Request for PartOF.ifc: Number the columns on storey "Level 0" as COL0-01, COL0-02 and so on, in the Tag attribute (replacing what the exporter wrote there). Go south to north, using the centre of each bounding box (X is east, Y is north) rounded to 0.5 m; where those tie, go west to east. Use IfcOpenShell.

First a look at what the model holds.

```python
import ifcopenshell
import ifcopenshell.util.element
import ifcopenshell.util.placement

model = ifcopenshell.open("PartOF.ifc")
print(model.schema)
storey = next(s for s in model.by_type("IfcBuildingStorey") if s.Name == "Level 0")
columns = [e for e in ifcopenshell.util.element.get_decomposition(storey) if e.is_a("IfcColumn")]
for e in sorted(columns, key=lambda e: e.id()):
    origin = ifcopenshell.util.placement.get_local_placement(e.ObjectPlacement)[:3, 3]
    print(e.id(), e.Tag, e.Name, origin.round(2) + 0.0, sep=" | ")
```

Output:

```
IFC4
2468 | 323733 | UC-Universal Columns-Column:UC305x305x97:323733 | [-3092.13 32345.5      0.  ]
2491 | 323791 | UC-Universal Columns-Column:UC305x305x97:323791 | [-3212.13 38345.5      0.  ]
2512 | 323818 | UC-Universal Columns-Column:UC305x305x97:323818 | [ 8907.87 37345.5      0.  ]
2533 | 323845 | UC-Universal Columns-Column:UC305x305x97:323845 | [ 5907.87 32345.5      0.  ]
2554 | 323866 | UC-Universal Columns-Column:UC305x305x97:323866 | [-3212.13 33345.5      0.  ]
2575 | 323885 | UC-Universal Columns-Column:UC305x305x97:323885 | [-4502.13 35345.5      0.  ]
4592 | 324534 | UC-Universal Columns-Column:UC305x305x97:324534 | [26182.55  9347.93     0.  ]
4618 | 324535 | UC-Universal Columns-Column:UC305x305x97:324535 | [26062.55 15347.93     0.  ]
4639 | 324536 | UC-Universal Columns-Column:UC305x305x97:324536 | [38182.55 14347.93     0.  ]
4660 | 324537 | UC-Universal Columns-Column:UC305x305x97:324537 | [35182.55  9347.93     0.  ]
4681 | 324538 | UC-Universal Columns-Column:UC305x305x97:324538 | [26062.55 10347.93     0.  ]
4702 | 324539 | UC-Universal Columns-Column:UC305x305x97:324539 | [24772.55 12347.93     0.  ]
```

```python
import ifcopenshell
import ifcopenshell.geom
import ifcopenshell.util.element
import ifcopenshell.util.shape

model = ifcopenshell.open("PartOF.ifc")
settings = ifcopenshell.geom.settings()
settings.set("use-world-coords", True)


def centre(element):
    shape = ifcopenshell.geom.create_shape(settings, element)
    return ifcopenshell.util.shape.get_bbox_centroid(shape.geometry)


storey = next(s for s in model.by_type("IfcBuildingStorey") if s.Name == "Level 0")
columns = [e for e in ifcopenshell.util.element.get_decomposition(storey) if e.is_a("IfcColumn")]

# Insertion points can sit at a corner or the storey origin, so sort by the geometry (in metres).
centres = {e: centre(e) for e in columns}
columns.sort(key=lambda e: (round(centres[e][1] / 0.5), centres[e][0]))

for i, e in enumerate(columns, start=1):
    number = f"COL0-{i:02d}"
    e.Tag = number
    print(e.id(), number)

model.write("PartOF_updated.ifc")
```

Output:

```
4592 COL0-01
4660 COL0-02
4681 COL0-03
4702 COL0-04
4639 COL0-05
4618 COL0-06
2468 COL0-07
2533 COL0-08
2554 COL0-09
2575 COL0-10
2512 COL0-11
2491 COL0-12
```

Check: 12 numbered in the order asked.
